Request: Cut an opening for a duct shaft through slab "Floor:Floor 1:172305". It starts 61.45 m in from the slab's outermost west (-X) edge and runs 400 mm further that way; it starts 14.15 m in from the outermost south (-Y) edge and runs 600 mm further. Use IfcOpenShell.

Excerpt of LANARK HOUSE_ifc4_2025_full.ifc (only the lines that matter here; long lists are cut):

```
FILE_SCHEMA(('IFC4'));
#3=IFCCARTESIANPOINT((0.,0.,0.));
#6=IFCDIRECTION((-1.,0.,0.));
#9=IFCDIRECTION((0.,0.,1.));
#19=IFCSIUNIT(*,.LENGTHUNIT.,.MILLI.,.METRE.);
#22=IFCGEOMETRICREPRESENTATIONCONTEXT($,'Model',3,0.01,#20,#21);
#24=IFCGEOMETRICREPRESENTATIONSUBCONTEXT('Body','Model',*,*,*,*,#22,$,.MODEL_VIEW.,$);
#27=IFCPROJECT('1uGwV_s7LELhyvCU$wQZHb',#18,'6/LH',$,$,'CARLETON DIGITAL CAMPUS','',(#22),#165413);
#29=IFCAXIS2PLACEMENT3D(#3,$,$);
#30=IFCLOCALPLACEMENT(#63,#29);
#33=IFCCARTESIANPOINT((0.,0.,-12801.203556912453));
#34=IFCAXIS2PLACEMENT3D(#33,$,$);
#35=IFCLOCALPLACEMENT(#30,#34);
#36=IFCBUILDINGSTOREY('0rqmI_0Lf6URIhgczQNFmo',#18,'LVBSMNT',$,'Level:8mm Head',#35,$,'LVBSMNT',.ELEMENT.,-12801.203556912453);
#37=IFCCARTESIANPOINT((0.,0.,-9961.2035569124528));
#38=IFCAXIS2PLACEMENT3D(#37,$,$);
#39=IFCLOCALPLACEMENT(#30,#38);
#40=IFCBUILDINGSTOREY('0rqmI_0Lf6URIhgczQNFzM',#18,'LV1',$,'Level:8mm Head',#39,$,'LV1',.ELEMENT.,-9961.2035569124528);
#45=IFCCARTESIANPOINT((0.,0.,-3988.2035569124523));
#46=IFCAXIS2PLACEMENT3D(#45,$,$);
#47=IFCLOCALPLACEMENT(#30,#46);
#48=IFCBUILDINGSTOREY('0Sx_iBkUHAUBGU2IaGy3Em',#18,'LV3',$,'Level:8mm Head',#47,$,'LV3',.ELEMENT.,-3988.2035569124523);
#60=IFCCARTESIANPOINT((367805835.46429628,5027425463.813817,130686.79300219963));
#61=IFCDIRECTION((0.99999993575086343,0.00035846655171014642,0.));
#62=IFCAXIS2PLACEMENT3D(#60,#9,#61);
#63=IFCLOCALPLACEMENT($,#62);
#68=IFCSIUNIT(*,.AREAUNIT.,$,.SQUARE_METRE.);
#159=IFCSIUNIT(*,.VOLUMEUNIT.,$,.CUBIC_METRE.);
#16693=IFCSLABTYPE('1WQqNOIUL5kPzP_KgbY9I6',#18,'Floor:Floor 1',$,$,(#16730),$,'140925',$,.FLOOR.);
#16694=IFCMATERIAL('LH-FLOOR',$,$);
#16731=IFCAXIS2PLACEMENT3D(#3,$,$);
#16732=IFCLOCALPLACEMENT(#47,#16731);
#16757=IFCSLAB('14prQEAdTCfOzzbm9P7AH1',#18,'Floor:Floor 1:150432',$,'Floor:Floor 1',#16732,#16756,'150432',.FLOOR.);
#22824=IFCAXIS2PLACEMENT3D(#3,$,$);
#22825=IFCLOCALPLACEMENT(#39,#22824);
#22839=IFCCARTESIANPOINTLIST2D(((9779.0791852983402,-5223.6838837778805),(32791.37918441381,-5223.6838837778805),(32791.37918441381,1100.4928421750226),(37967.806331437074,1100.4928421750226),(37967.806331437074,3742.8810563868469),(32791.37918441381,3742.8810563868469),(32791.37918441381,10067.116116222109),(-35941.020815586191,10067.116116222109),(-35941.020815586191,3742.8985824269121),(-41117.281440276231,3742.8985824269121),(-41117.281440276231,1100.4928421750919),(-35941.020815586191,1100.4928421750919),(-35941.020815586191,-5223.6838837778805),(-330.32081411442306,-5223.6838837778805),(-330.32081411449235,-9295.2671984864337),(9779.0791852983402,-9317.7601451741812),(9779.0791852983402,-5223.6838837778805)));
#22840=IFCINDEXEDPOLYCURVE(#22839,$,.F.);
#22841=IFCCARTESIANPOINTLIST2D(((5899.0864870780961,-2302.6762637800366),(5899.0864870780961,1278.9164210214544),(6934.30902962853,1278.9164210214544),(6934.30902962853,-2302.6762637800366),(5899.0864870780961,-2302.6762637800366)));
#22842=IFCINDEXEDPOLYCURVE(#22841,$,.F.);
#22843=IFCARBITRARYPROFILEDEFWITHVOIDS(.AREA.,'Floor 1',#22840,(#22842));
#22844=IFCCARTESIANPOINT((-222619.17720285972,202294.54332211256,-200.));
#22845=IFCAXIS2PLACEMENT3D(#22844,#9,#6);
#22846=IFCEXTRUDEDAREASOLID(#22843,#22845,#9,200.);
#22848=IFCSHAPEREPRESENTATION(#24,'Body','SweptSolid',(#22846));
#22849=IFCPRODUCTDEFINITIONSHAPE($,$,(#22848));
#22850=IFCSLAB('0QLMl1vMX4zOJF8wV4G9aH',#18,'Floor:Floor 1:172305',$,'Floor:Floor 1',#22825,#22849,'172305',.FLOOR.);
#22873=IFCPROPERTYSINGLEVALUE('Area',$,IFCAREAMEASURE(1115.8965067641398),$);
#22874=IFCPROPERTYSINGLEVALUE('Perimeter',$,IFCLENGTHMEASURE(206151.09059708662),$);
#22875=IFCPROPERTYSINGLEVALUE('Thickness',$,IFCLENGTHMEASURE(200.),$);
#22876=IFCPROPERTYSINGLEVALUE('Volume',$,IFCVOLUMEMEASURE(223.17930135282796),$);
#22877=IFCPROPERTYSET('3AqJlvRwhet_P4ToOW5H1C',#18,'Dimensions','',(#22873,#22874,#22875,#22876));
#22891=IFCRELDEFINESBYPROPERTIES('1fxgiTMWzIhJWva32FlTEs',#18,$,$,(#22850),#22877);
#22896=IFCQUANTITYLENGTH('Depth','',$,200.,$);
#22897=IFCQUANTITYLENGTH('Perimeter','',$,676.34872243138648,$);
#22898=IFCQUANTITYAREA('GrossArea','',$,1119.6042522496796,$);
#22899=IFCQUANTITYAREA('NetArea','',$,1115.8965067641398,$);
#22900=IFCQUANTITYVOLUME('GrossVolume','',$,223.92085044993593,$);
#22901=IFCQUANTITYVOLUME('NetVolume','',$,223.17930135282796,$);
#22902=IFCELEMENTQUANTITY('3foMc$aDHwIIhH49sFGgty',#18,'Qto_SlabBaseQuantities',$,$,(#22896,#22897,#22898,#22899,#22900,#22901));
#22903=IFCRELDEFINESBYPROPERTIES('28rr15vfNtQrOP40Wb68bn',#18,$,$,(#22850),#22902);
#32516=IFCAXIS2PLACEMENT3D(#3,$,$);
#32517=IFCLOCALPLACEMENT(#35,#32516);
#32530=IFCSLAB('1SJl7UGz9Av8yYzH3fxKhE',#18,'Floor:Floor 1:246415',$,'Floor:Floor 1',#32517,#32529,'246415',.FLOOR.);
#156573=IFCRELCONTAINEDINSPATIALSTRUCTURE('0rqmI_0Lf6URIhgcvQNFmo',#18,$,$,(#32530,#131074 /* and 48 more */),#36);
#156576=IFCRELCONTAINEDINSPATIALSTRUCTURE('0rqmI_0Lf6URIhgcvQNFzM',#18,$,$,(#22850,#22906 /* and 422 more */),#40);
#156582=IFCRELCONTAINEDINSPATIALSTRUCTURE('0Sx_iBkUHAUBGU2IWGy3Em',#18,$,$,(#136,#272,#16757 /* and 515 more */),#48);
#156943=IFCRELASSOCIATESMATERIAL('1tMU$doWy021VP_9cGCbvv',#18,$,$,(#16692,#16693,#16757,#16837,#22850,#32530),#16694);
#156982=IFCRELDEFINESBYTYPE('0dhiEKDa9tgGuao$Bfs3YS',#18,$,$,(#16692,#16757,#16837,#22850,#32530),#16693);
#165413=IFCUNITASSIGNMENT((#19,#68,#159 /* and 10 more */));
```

```python
import numpy as np
import ifcopenshell
import ifcopenshell.api.feature
import ifcopenshell.api.geometry
import ifcopenshell.api.pset
import ifcopenshell.api.root
import ifcopenshell.geom
import ifcopenshell.util.element
import ifcopenshell.util.placement
import ifcopenshell.util.representation
import ifcopenshell.util.shape
import ifcopenshell.util.unit

model = ifcopenshell.open("LANARK HOUSE_ifc4_2025_full.ifc")
unit_scale = ifcopenshell.util.unit.calculate_unit_scale(model)
area_scale = ifcopenshell.util.unit.calculate_unit_scale(model, "AREAUNIT")
volume_scale = ifcopenshell.util.unit.calculate_unit_scale(model, "VOLUMEUNIT")
settings = ifcopenshell.geom.settings()


def volume(element):
    """Net volume in cubic metres, openings subtracted."""
    shape = ifcopenshell.geom.create_shape(settings, element)
    return ifcopenshell.util.shape.get_volume(shape.geometry)


slab = model.by_guid("0QLMl1vMX4zOJF8wV4G9aH")
before = volume(slab)

# Extent in the slab's own axes, in metres. The edges named are its -X and -Y sides.
slab_shape = ifcopenshell.geom.create_shape(settings, slab)
vertices = ifcopenshell.util.shape.get_vertices(slab_shape.geometry)
x_min, y_min, bottom = vertices.min(axis=0)
top = vertices[:, 2].max()

opening = ifcopenshell.api.root.create_entity(model, ifc_class="IfcOpeningElement", name="Duct shaft opening", predefined_type="OPENING")
context = ifcopenshell.util.representation.get_context(model, "Model", "Body", "MODEL_VIEW")
width, depth = 0.4, 0.6
outline = [(0.0, 0.0), (width, 0.0), (width, depth), (0.0, depth), (0.0, 0.0)]
# Overshoot both faces by 50 mm so the cut is clean.
shape = ifcopenshell.api.geometry.add_slab_representation(
    model, context=context, depth=top - bottom + 0.1, polyline=outline
)
ifcopenshell.api.geometry.assign_representation(model, product=opening, representation=shape)

matrix = ifcopenshell.util.placement.get_local_placement(slab.ObjectPlacement)
matrix[:, 3] = matrix @ np.append(np.array([x_min + 61.45, y_min + 14.15, bottom - 0.05]) / unit_scale, 1.0)
ifcopenshell.api.geometry.edit_object_placement(model, product=opening, matrix=matrix, is_si=False)
ifcopenshell.api.feature.add_feature(model, feature=opening, element=slab)

after = volume(slab)

# Update the slab's stored quantities.
pset = model.by_id(ifcopenshell.util.element.get_pset(slab, "Dimensions", should_inherit=False)["id"])
ifcopenshell.api.pset.edit_pset(model, pset=pset, properties={
    "Area": model.create_entity("IfcAreaMeasure", after / (top - bottom) / area_scale),
    "Volume": model.create_entity("IfcVolumeMeasure", after / volume_scale),
})
qto = model.by_id(ifcopenshell.util.element.get_pset(slab, "Qto_SlabBaseQuantities", should_inherit=False)["id"])
ifcopenshell.api.pset.edit_qto(model, qto=qto, properties={
    "NetArea": after / (top - bottom) / area_scale,
    "NetVolume": after / volume_scale,
})

print(f"slab volume {before:.3f} -> {after:.3f} m3")

model.write("LANARK HOUSE_ifc4_2025_full-out.ifc")
```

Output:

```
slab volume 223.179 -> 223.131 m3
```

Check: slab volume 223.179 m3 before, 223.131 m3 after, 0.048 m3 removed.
